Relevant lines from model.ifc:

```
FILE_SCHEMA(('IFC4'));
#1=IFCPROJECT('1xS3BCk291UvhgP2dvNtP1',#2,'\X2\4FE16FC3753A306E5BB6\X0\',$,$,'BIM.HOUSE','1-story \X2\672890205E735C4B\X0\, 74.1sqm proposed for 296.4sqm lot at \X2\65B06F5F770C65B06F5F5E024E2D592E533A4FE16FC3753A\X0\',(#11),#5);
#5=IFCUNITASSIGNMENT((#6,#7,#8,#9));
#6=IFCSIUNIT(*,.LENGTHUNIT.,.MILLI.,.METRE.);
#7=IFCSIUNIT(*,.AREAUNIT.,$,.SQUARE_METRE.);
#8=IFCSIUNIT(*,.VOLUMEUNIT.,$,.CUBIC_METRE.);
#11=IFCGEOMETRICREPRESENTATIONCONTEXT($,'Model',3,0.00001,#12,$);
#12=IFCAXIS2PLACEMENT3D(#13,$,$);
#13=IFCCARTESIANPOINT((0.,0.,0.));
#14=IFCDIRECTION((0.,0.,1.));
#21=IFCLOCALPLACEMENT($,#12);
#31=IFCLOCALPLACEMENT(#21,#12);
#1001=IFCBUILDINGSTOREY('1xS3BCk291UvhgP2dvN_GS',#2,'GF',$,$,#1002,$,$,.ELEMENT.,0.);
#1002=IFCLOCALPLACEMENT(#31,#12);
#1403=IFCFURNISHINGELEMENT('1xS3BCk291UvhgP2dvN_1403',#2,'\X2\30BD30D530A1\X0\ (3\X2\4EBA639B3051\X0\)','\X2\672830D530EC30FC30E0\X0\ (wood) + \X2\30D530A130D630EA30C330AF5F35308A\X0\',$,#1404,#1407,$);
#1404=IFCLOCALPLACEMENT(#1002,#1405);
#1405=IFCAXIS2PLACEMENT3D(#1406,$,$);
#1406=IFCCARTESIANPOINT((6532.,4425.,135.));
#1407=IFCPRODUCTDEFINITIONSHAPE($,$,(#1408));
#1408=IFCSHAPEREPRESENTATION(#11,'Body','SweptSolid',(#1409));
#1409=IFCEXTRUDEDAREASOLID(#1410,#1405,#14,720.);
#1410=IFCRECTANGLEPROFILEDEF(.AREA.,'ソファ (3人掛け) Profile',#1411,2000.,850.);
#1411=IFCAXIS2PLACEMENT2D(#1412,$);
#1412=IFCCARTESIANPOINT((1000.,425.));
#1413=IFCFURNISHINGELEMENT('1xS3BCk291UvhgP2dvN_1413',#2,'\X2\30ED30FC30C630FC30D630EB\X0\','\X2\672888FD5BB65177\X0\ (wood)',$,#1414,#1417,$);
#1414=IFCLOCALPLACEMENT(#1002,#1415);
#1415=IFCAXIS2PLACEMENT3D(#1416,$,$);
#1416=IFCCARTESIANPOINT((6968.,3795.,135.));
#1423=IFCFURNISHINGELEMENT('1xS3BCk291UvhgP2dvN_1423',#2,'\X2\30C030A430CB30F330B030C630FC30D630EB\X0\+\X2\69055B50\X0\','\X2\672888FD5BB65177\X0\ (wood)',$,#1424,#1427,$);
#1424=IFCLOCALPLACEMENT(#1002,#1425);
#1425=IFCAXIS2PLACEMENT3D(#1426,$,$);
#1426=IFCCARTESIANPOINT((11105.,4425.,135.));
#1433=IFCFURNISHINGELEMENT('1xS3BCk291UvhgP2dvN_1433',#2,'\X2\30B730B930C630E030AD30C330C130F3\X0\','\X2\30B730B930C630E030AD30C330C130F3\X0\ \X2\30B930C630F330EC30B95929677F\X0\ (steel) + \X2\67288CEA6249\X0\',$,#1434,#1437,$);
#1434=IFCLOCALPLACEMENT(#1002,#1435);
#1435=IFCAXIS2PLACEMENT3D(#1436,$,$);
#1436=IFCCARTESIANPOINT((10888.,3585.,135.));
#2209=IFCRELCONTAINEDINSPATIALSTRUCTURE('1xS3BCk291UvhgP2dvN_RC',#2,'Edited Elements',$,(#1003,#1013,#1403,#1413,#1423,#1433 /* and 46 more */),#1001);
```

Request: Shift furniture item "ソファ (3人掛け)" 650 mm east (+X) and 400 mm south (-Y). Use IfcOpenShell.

```python
import ifcopenshell
import ifcopenshell.api.geometry
import ifcopenshell.util.placement

model = ifcopenshell.open("model.ifc")

item = model.by_guid("1xS3BCk291UvhgP2dvN_1403")
matrix = ifcopenshell.util.placement.get_local_placement(item.ObjectPlacement)
matrix[0, 3] += 650.0
matrix[1, 3] -= 400.0
ifcopenshell.api.geometry.edit_object_placement(model, product=item, matrix=matrix, is_si=False)

print(ifcopenshell.util.placement.get_local_placement(item.ObjectPlacement).round(3) + 0.0)

model.write("model_edited.ifc")
```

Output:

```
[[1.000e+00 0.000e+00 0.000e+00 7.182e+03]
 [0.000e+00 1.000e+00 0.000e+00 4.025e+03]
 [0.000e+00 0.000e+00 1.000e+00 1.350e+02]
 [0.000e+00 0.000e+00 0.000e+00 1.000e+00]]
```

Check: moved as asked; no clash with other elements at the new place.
